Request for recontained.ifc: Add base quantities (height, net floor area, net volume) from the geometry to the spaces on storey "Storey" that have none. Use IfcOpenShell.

First a look at what the model holds.

```python
import ifcopenshell
import ifcopenshell.util.element
import ifcopenshell.util.unit

model = ifcopenshell.open("recontained.ifc")
print(model.schema)
for unit_type in ("LENGTHUNIT", "AREAUNIT", "VOLUMEUNIT"):
    print(unit_type, ifcopenshell.util.unit.calculate_unit_scale(model, unit_type))
storey = next(s for s in model.by_type("IfcBuildingStorey") if s.Name == "Storey")
spaces = [e for e in ifcopenshell.util.element.get_decomposition(storey) if e.is_a("IfcSpace")]
for e in sorted(spaces, key=lambda e: e.id()):
    print(e.id(), e.is_a(), e.Name, list(ifcopenshell.util.element.get_psets(e, qtos_only=True)), sep=" | ")
```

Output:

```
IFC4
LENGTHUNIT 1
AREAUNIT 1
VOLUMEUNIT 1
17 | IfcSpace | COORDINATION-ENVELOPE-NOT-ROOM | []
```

```python
import ifcopenshell
import ifcopenshell.api.pset
import ifcopenshell.geom
import ifcopenshell.util.element
import ifcopenshell.util.shape
import ifcopenshell.util.unit

model = ifcopenshell.open("recontained.ifc")
unit_scale = ifcopenshell.util.unit.calculate_unit_scale(model)
area_scale = ifcopenshell.util.unit.calculate_unit_scale(model, "AREAUNIT")
volume_scale = ifcopenshell.util.unit.calculate_unit_scale(model, "VOLUMEUNIT")
settings = ifcopenshell.geom.settings()

storey = next(s for s in model.by_type("IfcBuildingStorey") if s.Name == "Storey")
spaces = [e for e in ifcopenshell.util.element.get_decomposition(storey) if e.is_a("IfcSpace")]

for e in sorted(spaces, key=lambda e: e.id()):
    if ifcopenshell.util.element.get_psets(e, qtos_only=True, should_inherit=False):
        continue
    # Geometry comes back in metres, in the element's own axes.
    shape = ifcopenshell.geom.create_shape(settings, e)
    values = {
        "Height": ifcopenshell.util.shape.get_z(shape.geometry) / unit_scale,
        "NetFloorArea": ifcopenshell.util.shape.get_footprint_area(shape.geometry) / area_scale,
        "NetVolume": ifcopenshell.util.shape.get_volume(shape.geometry) / volume_scale,
    }
    qto = ifcopenshell.api.pset.add_qto(model, product=e, name="Qto_SpaceBaseQuantities")
    ifcopenshell.api.pset.edit_qto(model, qto=qto, properties=values)
    print(e.id(), {k: round(v, 3) for k, v in values.items()})

model.write("recontained_rev.ifc")
```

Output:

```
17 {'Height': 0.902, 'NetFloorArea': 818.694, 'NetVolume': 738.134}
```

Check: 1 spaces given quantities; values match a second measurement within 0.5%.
